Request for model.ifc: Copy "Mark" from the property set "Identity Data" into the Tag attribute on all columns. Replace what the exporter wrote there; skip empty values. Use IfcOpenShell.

First a look at what the model holds.

```python
import ifcopenshell
import ifcopenshell.util.element

model = ifcopenshell.open("model.ifc")
print(model.schema)
columns = model.by_type("IfcColumn")
print(len(columns), "columns")
for e in columns[:8]:
    source = ifcopenshell.util.element.get_pset(e, "Identity Data", "Mark")
    target = e.Tag
    print(e.id(), repr(source), repr(target), sep=" | ")
```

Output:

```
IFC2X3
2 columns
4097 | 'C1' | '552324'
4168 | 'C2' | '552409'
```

```python
import ifcopenshell
import ifcopenshell.util.element

model = ifcopenshell.open("model.ifc")

count = 0
for e in model.by_type("IfcColumn"):
    value = ifcopenshell.util.element.get_pset(e, "Identity Data", "Mark")
    current = e.Tag
    if not value or not value.strip() or current == value:
        continue
    e.Tag = value
    count += 1

print(count, "columns updated")

model.write("model_rev.ifc")
```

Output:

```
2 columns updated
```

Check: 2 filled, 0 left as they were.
